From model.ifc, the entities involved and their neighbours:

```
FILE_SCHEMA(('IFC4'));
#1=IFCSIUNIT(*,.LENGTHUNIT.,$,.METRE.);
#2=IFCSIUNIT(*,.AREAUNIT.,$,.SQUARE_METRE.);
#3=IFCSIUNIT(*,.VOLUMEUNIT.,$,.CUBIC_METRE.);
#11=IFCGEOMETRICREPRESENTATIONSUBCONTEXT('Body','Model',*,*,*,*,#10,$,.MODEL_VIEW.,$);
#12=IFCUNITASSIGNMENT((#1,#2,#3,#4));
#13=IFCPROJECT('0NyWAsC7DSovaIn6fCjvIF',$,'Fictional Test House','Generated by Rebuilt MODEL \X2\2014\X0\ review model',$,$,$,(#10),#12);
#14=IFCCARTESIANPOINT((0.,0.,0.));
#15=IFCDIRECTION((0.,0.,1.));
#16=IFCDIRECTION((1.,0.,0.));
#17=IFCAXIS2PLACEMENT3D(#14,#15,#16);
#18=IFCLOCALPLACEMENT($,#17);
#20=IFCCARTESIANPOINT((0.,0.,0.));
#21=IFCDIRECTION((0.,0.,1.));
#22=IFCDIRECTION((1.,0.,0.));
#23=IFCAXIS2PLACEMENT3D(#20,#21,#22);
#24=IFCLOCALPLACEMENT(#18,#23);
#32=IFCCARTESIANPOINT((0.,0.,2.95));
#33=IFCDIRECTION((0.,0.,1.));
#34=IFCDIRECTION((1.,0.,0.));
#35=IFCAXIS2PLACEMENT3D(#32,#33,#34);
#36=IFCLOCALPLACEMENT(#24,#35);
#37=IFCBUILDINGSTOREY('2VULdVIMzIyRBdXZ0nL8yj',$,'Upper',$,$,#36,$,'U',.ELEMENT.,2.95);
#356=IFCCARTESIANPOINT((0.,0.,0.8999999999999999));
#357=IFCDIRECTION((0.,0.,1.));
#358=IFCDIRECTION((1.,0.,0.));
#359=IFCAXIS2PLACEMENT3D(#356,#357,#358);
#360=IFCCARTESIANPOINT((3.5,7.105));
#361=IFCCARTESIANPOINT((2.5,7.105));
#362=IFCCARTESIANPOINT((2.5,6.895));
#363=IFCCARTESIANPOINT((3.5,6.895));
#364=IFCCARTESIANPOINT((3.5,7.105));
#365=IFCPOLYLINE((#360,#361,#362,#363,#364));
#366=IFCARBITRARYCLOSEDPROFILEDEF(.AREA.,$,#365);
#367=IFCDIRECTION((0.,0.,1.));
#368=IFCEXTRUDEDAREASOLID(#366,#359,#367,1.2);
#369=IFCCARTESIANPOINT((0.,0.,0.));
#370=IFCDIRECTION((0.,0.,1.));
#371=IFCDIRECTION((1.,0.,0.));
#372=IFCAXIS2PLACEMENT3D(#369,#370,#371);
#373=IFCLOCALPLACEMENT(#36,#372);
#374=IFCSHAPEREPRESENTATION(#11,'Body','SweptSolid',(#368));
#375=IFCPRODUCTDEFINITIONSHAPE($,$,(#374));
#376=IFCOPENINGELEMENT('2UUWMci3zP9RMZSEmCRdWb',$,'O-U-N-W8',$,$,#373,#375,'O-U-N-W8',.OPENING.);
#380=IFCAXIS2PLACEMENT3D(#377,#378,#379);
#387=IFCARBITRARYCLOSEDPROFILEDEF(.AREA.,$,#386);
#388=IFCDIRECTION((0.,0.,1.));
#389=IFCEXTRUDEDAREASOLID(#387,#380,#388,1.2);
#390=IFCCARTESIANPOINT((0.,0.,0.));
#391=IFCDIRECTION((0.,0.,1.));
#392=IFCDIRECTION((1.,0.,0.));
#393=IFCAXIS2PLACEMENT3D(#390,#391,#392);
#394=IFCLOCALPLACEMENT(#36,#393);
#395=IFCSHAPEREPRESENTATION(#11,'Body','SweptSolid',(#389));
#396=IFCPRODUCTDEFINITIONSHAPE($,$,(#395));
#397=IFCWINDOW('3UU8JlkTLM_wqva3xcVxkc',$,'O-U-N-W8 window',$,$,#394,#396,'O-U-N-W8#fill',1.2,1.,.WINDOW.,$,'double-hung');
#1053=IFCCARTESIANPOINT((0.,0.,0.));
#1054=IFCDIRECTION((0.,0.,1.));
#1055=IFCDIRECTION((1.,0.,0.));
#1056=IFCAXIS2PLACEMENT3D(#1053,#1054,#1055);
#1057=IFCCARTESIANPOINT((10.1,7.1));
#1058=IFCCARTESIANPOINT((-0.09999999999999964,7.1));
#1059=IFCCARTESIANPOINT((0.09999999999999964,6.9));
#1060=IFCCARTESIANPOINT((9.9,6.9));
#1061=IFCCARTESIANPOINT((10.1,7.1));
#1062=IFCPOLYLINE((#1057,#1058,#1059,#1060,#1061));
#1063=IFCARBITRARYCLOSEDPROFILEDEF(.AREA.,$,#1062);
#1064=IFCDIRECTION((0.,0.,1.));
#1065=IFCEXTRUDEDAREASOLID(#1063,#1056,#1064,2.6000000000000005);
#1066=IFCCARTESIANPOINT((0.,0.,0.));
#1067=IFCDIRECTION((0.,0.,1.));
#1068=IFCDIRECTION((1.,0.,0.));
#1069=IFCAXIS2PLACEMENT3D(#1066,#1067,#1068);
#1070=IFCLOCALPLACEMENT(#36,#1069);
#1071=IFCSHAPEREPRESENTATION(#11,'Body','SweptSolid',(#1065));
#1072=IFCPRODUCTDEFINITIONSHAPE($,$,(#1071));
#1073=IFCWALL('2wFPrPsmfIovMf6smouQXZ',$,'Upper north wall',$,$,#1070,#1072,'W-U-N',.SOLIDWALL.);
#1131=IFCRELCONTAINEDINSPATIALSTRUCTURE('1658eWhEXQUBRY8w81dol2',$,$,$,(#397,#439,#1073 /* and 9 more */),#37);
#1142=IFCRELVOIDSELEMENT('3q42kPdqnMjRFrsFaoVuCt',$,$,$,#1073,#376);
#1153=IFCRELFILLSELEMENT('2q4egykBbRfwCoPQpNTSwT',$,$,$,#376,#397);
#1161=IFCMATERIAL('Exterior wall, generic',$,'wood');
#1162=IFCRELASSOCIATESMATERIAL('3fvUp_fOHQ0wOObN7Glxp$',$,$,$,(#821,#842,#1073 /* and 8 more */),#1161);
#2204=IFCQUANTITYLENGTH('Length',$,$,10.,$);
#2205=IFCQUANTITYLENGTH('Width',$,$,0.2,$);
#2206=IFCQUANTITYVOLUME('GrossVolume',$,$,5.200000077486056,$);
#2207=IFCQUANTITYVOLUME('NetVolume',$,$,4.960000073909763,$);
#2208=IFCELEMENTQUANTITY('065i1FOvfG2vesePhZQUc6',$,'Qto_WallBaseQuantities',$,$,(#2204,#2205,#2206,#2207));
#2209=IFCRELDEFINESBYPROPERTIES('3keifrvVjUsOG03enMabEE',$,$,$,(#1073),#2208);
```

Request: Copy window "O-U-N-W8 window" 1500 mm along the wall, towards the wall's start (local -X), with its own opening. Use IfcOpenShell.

```python
import ifcopenshell
import ifcopenshell.api.feature
import ifcopenshell.api.geometry
import ifcopenshell.api.pset
import ifcopenshell.api.root
import ifcopenshell.geom
import ifcopenshell.util.element
import ifcopenshell.util.placement
import ifcopenshell.util.shape
import ifcopenshell.util.unit

model = ifcopenshell.open("model.ifc")
unit_scale = ifcopenshell.util.unit.calculate_unit_scale(model)
volume_scale = ifcopenshell.util.unit.calculate_unit_scale(model, "VOLUMEUNIT")
settings = ifcopenshell.geom.settings()


def volume(element):
    """Net volume in cubic metres, openings subtracted."""
    shape = ifcopenshell.geom.create_shape(settings, element)
    return ifcopenshell.util.shape.get_volume(shape.geometry)


window = model.by_guid("3UU8JlkTLM_wqva3xcVxkc")
opening = window.FillsVoids[0].RelatingOpeningElement
wall = opening.VoidsElements[0].RelatingBuildingElement
before = volume(wall)
shift = ifcopenshell.util.placement.get_local_placement(wall.ObjectPlacement)[:3, 0] * -1.5 / unit_scale

# copy_class copies the void relationship, type, container and properties, but no geometry.
new_opening = ifcopenshell.api.root.copy_class(model, product=opening)
new_opening.Representation = ifcopenshell.util.element.copy_deep(
    model, opening.Representation, exclude=["IfcGeometricRepresentationContext", "IfcRepresentationMap"]
)
new_opening.Tag = None
new_window = ifcopenshell.api.root.copy_class(model, product=window)
new_window.Representation = ifcopenshell.util.element.copy_deep(
    model, window.Representation, exclude=["IfcGeometricRepresentationContext", "IfcRepresentationMap"]
)
new_window.Tag = None
ifcopenshell.api.feature.add_filling(model, opening=new_opening, element=new_window)

for old, new in ((opening, new_opening), (window, new_window)):
    matrix = ifcopenshell.util.placement.get_local_placement(old.ObjectPlacement)
    matrix[:3, 3] += shift
    ifcopenshell.api.geometry.edit_object_placement(model, product=new, matrix=matrix, is_si=False)

after = volume(wall)

# Update the wall's stored quantities.
qto = model.by_id(ifcopenshell.util.element.get_pset(wall, "Qto_WallBaseQuantities", should_inherit=False)["id"])
ifcopenshell.api.pset.edit_qto(model, qto=qto, properties={"NetVolume": after / volume_scale})

print(f"wall volume {before:.3f} -> {after:.3f} m3")

model.write("model_v2.ifc")
```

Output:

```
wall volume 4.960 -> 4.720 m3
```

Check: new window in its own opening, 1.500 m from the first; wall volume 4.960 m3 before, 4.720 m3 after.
